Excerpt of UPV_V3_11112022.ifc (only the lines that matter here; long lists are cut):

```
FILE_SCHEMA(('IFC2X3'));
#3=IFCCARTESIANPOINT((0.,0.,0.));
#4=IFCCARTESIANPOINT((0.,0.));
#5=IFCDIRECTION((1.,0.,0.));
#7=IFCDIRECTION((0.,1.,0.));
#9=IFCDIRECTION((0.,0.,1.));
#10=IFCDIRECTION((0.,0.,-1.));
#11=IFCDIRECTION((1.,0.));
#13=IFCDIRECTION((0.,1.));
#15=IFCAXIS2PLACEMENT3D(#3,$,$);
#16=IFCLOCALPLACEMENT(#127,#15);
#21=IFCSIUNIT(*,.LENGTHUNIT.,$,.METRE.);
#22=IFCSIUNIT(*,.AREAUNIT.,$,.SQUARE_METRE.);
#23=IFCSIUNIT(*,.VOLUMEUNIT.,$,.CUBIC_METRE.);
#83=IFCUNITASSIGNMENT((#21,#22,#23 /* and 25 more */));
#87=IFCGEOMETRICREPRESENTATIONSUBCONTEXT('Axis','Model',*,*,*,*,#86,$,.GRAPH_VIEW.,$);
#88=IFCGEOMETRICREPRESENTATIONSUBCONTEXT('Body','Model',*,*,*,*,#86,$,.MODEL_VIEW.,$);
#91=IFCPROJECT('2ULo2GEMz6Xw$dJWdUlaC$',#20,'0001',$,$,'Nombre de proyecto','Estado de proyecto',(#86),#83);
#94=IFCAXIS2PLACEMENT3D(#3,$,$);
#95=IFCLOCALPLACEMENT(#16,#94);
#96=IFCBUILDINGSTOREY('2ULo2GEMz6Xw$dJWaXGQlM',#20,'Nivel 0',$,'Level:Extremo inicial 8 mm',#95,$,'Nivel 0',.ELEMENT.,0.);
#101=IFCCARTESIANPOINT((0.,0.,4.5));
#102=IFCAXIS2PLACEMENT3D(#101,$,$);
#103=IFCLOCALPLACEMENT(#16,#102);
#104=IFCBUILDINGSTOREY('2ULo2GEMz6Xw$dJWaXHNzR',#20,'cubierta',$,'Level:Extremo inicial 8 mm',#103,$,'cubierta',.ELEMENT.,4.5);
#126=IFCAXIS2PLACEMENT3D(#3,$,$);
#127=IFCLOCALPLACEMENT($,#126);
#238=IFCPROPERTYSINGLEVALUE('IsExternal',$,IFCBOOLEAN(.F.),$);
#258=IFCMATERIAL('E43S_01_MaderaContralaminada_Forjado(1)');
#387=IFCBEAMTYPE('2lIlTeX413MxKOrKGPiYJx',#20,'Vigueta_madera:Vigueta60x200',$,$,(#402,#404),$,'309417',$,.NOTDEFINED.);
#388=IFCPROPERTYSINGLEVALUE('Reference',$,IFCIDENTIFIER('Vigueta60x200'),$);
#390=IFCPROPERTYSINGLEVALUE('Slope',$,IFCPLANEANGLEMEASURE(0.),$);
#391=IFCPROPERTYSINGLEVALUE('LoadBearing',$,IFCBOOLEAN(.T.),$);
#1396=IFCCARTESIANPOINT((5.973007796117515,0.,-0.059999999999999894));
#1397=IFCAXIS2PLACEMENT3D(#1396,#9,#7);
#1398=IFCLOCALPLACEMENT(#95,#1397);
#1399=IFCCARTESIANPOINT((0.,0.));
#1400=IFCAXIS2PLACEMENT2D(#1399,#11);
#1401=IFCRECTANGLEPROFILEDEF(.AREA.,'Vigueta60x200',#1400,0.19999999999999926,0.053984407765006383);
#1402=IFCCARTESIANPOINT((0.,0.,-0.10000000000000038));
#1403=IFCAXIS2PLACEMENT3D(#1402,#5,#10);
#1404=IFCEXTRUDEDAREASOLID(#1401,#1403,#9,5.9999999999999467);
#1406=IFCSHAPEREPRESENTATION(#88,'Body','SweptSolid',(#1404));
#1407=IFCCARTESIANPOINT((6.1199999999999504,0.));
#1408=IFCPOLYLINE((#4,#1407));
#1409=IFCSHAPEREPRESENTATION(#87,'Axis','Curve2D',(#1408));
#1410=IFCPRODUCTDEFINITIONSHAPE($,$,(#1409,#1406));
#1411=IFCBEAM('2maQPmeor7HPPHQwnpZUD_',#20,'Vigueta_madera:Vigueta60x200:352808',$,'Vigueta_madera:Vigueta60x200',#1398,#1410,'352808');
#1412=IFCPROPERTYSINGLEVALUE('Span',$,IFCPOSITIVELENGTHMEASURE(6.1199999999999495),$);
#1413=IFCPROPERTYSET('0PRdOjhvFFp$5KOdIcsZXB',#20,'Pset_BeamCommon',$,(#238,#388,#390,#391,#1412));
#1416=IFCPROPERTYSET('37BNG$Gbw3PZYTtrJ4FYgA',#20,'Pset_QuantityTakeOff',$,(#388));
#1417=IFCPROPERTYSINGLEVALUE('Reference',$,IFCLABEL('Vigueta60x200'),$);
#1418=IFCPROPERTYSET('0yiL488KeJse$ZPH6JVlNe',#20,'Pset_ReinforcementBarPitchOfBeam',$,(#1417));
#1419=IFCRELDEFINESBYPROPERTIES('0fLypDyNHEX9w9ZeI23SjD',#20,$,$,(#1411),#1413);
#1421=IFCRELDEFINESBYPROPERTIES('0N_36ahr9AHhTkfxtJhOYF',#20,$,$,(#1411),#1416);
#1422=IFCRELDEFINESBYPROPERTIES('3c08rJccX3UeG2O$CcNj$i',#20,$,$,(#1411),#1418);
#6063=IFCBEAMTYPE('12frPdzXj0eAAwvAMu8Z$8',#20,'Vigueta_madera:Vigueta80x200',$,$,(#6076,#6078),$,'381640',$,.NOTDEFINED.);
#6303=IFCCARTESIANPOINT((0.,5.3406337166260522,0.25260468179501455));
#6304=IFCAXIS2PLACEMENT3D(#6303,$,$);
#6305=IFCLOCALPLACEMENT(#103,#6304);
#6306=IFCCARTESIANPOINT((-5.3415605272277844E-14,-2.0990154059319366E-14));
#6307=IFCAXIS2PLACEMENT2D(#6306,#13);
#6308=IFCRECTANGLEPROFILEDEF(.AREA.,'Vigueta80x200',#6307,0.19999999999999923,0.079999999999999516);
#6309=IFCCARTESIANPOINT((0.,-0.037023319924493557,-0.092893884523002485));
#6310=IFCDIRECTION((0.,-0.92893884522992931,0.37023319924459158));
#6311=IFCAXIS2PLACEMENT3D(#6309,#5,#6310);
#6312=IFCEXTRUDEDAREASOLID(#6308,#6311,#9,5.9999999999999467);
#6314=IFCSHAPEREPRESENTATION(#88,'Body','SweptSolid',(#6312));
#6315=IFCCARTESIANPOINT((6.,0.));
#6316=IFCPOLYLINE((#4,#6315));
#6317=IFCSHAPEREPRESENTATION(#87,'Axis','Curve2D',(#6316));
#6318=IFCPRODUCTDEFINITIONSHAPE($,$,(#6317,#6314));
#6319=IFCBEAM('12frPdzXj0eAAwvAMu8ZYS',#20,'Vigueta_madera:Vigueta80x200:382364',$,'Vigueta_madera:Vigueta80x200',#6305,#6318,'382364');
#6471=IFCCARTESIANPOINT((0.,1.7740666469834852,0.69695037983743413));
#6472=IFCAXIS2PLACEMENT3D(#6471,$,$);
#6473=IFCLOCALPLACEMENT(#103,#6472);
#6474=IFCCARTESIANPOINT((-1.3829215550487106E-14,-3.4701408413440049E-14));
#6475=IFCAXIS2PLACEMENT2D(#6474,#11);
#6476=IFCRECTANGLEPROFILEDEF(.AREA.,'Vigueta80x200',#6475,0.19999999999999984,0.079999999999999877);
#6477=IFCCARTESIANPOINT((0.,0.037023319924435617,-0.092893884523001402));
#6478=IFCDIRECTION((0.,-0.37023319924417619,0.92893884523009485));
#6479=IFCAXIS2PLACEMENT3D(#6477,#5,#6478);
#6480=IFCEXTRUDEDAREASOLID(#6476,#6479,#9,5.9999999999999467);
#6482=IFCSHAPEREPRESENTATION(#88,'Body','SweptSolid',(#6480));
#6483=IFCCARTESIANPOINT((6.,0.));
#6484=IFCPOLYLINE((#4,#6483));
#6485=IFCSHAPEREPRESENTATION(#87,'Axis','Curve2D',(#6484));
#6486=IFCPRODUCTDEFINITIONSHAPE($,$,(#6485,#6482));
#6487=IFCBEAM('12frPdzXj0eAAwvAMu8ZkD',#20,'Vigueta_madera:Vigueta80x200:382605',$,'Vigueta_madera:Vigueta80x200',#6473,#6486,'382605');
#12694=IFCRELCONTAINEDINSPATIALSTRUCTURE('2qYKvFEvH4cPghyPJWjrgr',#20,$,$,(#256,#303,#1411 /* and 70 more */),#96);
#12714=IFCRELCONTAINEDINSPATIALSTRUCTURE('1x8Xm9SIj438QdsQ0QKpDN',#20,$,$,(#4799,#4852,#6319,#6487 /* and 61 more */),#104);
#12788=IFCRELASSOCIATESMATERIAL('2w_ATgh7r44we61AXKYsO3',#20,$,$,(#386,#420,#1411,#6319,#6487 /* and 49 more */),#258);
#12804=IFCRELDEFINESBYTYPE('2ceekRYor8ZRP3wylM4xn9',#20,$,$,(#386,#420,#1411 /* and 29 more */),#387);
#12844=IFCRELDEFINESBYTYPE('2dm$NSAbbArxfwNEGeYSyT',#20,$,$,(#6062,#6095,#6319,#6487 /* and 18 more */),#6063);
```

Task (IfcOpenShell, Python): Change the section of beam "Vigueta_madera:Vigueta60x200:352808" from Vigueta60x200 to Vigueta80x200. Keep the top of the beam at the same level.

```python
import ifcopenshell
import ifcopenshell.api.pset
import ifcopenshell.api.type
import ifcopenshell.util.element
import ifcopenshell.util.representation

model = ifcopenshell.open("UPV_V3_11112022.ifc")

member = model.by_guid("2maQPmeor7HPPHQwnpZUD_")
source = next(p for p in model.by_type("IfcRectangleProfileDef") if p.ProfileName == "Vigueta80x200")

body = ifcopenshell.util.representation.get_representation(member, "Model", "Body")
solid = body.Items[0]
old_profile = solid.SweptArea

# Copy the section's sizes but keep this member's own profile position.
profile = ifcopenshell.util.element.copy(model, source)
# Profiles are centred, so shift by half the change in depth to hold the top.
shift = (old_profile.XDim - profile.XDim) / 2
x, y = old_profile.Position.Location.Coordinates
up = (-1.0, 0.0)  # upwards, in the solid's own plane
location = model.createIfcCartesianPoint((x + up[0] * shift, y + up[1] * shift))
profile.Position = model.createIfcAxis2Placement2D(location, old_profile.Position.RefDirection)
solid.SweptArea = profile
if not model.get_total_inverses(old_profile):
    ifcopenshell.util.element.remove_deep2(model, old_profile)

new_type = model.by_guid("12frPdzXj0eAAwvAMu8Z$8")
ifcopenshell.api.type.assign_type(
    model, related_objects=[member], relating_type=new_type, should_map_representations=False
)
member.Name = member.Name.replace("Vigueta60x200", "Vigueta80x200")
member.ObjectType = "Vigueta_madera:Vigueta80x200"
pset = model.by_id(ifcopenshell.util.element.get_pset(member, "Pset_BeamCommon", should_inherit=False)["id"])
ifcopenshell.api.pset.edit_pset(model, pset=pset, properties={"Reference": "Vigueta80x200"})
pset = model.by_id(ifcopenshell.util.element.get_pset(member, "Pset_QuantityTakeOff", should_inherit=False)["id"])
ifcopenshell.api.pset.edit_pset(model, pset=pset, properties={"Reference": "Vigueta80x200"})
pset = model.by_id(ifcopenshell.util.element.get_pset(member, "Pset_ReinforcementBarPitchOfBeam", should_inherit=False)["id"])
ifcopenshell.api.pset.edit_pset(model, pset=pset, properties={"Reference": "Vigueta80x200"})

print(solid.SweptArea)

model.write("UPV_V3_11112022-out.ifc")
```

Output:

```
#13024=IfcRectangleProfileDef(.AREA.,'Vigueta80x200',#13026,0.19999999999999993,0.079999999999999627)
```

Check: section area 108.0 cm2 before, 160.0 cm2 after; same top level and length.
